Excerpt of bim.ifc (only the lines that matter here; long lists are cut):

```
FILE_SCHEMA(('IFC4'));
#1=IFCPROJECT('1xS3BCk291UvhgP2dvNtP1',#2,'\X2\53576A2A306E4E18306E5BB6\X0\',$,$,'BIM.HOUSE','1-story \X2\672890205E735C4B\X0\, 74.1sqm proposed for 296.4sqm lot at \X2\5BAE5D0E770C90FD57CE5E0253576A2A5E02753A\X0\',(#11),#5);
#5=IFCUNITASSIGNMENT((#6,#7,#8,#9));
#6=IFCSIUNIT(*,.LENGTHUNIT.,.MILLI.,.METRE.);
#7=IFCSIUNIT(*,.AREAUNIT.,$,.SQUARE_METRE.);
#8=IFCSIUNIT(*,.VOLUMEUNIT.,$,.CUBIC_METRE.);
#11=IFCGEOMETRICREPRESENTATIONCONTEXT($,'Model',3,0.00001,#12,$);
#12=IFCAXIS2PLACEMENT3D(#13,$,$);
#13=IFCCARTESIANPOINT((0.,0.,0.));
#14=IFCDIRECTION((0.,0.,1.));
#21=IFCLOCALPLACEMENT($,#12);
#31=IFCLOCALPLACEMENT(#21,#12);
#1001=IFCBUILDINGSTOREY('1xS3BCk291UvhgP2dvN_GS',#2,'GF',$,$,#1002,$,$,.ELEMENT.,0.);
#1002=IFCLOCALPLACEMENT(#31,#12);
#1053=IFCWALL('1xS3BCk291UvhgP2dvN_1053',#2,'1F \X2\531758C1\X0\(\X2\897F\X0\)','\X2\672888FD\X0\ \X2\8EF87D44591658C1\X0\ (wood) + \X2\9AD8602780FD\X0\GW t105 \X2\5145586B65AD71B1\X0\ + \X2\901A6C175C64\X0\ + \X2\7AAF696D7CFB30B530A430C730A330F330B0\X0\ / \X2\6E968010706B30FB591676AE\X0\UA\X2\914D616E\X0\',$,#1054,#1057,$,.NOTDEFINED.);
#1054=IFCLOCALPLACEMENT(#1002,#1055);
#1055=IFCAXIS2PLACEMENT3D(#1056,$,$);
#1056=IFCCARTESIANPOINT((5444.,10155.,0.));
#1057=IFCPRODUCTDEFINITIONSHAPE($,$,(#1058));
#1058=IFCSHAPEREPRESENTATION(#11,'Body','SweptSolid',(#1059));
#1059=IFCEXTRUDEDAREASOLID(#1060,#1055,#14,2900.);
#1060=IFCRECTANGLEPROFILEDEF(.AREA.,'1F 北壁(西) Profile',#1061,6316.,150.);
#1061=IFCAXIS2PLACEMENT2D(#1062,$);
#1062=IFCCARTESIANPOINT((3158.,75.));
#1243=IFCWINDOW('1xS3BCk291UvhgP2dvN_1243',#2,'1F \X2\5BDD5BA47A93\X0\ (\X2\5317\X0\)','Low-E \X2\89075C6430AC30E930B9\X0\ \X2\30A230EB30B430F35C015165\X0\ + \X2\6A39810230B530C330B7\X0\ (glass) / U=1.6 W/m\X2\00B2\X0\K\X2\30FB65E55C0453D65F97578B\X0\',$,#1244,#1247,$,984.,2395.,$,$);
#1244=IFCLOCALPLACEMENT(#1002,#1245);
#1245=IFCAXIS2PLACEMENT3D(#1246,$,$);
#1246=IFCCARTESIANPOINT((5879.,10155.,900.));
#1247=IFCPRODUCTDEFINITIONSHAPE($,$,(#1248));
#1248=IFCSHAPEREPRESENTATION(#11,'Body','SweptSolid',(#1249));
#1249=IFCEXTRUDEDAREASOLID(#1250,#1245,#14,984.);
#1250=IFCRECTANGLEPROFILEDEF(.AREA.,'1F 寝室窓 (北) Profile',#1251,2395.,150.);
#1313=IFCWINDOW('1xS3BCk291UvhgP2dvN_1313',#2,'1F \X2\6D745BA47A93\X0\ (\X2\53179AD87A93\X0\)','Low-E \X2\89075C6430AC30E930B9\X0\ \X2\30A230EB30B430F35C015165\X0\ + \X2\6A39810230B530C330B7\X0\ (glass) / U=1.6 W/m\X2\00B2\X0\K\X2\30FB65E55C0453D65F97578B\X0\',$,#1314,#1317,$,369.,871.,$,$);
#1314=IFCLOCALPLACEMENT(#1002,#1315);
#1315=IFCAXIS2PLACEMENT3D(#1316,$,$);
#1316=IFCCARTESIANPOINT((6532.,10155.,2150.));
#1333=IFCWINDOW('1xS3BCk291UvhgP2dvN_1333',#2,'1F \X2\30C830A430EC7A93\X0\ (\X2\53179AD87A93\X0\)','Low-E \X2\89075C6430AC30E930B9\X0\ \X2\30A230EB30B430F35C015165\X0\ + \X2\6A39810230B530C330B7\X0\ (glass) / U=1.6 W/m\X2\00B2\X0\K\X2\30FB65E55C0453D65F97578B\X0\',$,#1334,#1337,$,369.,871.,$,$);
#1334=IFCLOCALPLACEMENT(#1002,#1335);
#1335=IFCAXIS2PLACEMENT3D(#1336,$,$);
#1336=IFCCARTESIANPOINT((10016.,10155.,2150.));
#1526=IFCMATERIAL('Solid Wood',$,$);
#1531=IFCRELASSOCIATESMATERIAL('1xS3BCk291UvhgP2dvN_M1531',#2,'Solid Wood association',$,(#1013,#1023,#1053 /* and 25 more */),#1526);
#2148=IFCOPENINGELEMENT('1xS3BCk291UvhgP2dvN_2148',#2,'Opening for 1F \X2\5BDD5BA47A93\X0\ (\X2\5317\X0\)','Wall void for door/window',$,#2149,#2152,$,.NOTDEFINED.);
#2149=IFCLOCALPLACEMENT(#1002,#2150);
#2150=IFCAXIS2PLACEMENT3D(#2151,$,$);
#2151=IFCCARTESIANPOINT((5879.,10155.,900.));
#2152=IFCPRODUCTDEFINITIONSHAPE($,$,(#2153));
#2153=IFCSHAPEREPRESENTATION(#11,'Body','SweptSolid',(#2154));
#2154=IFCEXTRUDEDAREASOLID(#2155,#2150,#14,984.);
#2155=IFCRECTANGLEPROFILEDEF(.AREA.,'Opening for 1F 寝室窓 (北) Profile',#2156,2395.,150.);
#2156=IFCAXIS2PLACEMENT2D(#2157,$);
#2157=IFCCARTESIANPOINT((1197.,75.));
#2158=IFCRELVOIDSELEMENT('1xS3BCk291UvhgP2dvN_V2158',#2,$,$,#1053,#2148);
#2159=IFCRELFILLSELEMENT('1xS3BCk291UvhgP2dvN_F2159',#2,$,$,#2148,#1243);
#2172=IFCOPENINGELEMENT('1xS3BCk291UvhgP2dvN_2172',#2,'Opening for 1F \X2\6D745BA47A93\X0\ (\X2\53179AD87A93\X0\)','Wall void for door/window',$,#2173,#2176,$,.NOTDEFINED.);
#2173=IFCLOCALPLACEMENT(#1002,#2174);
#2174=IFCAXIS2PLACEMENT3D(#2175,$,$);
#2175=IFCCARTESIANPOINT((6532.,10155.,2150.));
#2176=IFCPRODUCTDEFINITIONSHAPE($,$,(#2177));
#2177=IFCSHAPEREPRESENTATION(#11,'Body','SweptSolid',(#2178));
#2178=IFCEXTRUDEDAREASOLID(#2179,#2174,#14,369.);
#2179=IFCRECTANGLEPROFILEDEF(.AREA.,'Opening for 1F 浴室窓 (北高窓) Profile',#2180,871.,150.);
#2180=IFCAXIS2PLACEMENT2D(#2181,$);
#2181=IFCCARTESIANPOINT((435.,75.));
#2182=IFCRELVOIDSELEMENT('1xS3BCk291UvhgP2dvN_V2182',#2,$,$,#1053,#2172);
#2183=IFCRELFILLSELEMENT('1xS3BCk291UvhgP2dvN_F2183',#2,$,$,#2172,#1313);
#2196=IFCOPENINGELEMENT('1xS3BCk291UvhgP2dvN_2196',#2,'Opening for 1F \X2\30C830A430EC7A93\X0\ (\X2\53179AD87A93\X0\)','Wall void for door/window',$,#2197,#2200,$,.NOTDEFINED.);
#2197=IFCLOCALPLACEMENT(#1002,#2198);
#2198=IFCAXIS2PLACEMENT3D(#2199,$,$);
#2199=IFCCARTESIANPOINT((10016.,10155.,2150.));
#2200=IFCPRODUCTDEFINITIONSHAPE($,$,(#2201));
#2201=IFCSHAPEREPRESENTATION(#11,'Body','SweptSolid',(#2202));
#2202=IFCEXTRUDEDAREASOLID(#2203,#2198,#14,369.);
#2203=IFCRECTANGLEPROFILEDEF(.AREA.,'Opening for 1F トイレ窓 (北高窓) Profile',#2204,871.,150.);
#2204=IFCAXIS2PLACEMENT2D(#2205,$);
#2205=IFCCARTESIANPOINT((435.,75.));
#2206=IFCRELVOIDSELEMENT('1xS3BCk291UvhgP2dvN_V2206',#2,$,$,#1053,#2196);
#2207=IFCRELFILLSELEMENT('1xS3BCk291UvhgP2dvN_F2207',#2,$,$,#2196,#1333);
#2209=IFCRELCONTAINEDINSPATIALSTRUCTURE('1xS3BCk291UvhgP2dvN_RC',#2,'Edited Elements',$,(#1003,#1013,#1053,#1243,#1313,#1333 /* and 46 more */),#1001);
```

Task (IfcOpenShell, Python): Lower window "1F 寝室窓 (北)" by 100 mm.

```python
import numpy as np
import ifcopenshell
import ifcopenshell.api.geometry
import ifcopenshell.util.placement
import ifcopenshell.util.unit

model = ifcopenshell.open("bim.ifc")
unit_scale = ifcopenshell.util.unit.calculate_unit_scale(model)

window = model.by_guid("1xS3BCk291UvhgP2dvN_1243")
opening = window.FillsVoids[0].RelatingOpeningElement
dz = -0.1 / unit_scale

shift = np.array([0.0, 0.0, dz])
# The window is not placed relative to its opening, so move both.
for product in (opening, window):
    matrix = ifcopenshell.util.placement.get_local_placement(product.ObjectPlacement)
    matrix[:3, 3] += shift
    ifcopenshell.api.geometry.edit_object_placement(model, product=product, matrix=matrix, is_si=False)

print(f"moved by {dz * unit_scale:+.3f} m")

model.write("bim_v2.ifc")
```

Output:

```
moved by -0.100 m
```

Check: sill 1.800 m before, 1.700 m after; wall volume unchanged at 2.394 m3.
